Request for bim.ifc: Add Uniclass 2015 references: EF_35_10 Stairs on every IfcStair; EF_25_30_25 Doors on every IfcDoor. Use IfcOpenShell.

First a look at what the model holds.

```python
import ifcopenshell

model = ifcopenshell.open("bim.ifc")
print(model.schema)
print("classifications:", [c.Name for c in model.by_type("IfcClassification")])
for ifc_class in ("IfcDoor", "IfcRoof", "IfcStair", "IfcWall", "IfcWindow"):
    print(ifc_class, len(model.by_type(ifc_class)))
```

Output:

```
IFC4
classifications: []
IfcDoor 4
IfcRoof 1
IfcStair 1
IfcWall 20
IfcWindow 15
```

```python
import ifcopenshell
import ifcopenshell.api.classification

model = ifcopenshell.open("bim.ifc")

system = ifcopenshell.api.classification.add_classification(model, classification="Uniclass 2015")

codes = {
    "IfcStair": ("EF_35_10", "Stairs"),
    "IfcDoor": ("EF_25_30_25", "Doors"),
}
for ifc_class, (code, name) in codes.items():
    products = model.by_type(ifc_class)
    ifcopenshell.api.classification.add_reference(
        model, products=products, classification=system, identification=code, name=name
    )
    print(code, len(products))

model.write("bim_updated.ifc")
```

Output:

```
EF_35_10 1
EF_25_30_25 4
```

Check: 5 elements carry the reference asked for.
